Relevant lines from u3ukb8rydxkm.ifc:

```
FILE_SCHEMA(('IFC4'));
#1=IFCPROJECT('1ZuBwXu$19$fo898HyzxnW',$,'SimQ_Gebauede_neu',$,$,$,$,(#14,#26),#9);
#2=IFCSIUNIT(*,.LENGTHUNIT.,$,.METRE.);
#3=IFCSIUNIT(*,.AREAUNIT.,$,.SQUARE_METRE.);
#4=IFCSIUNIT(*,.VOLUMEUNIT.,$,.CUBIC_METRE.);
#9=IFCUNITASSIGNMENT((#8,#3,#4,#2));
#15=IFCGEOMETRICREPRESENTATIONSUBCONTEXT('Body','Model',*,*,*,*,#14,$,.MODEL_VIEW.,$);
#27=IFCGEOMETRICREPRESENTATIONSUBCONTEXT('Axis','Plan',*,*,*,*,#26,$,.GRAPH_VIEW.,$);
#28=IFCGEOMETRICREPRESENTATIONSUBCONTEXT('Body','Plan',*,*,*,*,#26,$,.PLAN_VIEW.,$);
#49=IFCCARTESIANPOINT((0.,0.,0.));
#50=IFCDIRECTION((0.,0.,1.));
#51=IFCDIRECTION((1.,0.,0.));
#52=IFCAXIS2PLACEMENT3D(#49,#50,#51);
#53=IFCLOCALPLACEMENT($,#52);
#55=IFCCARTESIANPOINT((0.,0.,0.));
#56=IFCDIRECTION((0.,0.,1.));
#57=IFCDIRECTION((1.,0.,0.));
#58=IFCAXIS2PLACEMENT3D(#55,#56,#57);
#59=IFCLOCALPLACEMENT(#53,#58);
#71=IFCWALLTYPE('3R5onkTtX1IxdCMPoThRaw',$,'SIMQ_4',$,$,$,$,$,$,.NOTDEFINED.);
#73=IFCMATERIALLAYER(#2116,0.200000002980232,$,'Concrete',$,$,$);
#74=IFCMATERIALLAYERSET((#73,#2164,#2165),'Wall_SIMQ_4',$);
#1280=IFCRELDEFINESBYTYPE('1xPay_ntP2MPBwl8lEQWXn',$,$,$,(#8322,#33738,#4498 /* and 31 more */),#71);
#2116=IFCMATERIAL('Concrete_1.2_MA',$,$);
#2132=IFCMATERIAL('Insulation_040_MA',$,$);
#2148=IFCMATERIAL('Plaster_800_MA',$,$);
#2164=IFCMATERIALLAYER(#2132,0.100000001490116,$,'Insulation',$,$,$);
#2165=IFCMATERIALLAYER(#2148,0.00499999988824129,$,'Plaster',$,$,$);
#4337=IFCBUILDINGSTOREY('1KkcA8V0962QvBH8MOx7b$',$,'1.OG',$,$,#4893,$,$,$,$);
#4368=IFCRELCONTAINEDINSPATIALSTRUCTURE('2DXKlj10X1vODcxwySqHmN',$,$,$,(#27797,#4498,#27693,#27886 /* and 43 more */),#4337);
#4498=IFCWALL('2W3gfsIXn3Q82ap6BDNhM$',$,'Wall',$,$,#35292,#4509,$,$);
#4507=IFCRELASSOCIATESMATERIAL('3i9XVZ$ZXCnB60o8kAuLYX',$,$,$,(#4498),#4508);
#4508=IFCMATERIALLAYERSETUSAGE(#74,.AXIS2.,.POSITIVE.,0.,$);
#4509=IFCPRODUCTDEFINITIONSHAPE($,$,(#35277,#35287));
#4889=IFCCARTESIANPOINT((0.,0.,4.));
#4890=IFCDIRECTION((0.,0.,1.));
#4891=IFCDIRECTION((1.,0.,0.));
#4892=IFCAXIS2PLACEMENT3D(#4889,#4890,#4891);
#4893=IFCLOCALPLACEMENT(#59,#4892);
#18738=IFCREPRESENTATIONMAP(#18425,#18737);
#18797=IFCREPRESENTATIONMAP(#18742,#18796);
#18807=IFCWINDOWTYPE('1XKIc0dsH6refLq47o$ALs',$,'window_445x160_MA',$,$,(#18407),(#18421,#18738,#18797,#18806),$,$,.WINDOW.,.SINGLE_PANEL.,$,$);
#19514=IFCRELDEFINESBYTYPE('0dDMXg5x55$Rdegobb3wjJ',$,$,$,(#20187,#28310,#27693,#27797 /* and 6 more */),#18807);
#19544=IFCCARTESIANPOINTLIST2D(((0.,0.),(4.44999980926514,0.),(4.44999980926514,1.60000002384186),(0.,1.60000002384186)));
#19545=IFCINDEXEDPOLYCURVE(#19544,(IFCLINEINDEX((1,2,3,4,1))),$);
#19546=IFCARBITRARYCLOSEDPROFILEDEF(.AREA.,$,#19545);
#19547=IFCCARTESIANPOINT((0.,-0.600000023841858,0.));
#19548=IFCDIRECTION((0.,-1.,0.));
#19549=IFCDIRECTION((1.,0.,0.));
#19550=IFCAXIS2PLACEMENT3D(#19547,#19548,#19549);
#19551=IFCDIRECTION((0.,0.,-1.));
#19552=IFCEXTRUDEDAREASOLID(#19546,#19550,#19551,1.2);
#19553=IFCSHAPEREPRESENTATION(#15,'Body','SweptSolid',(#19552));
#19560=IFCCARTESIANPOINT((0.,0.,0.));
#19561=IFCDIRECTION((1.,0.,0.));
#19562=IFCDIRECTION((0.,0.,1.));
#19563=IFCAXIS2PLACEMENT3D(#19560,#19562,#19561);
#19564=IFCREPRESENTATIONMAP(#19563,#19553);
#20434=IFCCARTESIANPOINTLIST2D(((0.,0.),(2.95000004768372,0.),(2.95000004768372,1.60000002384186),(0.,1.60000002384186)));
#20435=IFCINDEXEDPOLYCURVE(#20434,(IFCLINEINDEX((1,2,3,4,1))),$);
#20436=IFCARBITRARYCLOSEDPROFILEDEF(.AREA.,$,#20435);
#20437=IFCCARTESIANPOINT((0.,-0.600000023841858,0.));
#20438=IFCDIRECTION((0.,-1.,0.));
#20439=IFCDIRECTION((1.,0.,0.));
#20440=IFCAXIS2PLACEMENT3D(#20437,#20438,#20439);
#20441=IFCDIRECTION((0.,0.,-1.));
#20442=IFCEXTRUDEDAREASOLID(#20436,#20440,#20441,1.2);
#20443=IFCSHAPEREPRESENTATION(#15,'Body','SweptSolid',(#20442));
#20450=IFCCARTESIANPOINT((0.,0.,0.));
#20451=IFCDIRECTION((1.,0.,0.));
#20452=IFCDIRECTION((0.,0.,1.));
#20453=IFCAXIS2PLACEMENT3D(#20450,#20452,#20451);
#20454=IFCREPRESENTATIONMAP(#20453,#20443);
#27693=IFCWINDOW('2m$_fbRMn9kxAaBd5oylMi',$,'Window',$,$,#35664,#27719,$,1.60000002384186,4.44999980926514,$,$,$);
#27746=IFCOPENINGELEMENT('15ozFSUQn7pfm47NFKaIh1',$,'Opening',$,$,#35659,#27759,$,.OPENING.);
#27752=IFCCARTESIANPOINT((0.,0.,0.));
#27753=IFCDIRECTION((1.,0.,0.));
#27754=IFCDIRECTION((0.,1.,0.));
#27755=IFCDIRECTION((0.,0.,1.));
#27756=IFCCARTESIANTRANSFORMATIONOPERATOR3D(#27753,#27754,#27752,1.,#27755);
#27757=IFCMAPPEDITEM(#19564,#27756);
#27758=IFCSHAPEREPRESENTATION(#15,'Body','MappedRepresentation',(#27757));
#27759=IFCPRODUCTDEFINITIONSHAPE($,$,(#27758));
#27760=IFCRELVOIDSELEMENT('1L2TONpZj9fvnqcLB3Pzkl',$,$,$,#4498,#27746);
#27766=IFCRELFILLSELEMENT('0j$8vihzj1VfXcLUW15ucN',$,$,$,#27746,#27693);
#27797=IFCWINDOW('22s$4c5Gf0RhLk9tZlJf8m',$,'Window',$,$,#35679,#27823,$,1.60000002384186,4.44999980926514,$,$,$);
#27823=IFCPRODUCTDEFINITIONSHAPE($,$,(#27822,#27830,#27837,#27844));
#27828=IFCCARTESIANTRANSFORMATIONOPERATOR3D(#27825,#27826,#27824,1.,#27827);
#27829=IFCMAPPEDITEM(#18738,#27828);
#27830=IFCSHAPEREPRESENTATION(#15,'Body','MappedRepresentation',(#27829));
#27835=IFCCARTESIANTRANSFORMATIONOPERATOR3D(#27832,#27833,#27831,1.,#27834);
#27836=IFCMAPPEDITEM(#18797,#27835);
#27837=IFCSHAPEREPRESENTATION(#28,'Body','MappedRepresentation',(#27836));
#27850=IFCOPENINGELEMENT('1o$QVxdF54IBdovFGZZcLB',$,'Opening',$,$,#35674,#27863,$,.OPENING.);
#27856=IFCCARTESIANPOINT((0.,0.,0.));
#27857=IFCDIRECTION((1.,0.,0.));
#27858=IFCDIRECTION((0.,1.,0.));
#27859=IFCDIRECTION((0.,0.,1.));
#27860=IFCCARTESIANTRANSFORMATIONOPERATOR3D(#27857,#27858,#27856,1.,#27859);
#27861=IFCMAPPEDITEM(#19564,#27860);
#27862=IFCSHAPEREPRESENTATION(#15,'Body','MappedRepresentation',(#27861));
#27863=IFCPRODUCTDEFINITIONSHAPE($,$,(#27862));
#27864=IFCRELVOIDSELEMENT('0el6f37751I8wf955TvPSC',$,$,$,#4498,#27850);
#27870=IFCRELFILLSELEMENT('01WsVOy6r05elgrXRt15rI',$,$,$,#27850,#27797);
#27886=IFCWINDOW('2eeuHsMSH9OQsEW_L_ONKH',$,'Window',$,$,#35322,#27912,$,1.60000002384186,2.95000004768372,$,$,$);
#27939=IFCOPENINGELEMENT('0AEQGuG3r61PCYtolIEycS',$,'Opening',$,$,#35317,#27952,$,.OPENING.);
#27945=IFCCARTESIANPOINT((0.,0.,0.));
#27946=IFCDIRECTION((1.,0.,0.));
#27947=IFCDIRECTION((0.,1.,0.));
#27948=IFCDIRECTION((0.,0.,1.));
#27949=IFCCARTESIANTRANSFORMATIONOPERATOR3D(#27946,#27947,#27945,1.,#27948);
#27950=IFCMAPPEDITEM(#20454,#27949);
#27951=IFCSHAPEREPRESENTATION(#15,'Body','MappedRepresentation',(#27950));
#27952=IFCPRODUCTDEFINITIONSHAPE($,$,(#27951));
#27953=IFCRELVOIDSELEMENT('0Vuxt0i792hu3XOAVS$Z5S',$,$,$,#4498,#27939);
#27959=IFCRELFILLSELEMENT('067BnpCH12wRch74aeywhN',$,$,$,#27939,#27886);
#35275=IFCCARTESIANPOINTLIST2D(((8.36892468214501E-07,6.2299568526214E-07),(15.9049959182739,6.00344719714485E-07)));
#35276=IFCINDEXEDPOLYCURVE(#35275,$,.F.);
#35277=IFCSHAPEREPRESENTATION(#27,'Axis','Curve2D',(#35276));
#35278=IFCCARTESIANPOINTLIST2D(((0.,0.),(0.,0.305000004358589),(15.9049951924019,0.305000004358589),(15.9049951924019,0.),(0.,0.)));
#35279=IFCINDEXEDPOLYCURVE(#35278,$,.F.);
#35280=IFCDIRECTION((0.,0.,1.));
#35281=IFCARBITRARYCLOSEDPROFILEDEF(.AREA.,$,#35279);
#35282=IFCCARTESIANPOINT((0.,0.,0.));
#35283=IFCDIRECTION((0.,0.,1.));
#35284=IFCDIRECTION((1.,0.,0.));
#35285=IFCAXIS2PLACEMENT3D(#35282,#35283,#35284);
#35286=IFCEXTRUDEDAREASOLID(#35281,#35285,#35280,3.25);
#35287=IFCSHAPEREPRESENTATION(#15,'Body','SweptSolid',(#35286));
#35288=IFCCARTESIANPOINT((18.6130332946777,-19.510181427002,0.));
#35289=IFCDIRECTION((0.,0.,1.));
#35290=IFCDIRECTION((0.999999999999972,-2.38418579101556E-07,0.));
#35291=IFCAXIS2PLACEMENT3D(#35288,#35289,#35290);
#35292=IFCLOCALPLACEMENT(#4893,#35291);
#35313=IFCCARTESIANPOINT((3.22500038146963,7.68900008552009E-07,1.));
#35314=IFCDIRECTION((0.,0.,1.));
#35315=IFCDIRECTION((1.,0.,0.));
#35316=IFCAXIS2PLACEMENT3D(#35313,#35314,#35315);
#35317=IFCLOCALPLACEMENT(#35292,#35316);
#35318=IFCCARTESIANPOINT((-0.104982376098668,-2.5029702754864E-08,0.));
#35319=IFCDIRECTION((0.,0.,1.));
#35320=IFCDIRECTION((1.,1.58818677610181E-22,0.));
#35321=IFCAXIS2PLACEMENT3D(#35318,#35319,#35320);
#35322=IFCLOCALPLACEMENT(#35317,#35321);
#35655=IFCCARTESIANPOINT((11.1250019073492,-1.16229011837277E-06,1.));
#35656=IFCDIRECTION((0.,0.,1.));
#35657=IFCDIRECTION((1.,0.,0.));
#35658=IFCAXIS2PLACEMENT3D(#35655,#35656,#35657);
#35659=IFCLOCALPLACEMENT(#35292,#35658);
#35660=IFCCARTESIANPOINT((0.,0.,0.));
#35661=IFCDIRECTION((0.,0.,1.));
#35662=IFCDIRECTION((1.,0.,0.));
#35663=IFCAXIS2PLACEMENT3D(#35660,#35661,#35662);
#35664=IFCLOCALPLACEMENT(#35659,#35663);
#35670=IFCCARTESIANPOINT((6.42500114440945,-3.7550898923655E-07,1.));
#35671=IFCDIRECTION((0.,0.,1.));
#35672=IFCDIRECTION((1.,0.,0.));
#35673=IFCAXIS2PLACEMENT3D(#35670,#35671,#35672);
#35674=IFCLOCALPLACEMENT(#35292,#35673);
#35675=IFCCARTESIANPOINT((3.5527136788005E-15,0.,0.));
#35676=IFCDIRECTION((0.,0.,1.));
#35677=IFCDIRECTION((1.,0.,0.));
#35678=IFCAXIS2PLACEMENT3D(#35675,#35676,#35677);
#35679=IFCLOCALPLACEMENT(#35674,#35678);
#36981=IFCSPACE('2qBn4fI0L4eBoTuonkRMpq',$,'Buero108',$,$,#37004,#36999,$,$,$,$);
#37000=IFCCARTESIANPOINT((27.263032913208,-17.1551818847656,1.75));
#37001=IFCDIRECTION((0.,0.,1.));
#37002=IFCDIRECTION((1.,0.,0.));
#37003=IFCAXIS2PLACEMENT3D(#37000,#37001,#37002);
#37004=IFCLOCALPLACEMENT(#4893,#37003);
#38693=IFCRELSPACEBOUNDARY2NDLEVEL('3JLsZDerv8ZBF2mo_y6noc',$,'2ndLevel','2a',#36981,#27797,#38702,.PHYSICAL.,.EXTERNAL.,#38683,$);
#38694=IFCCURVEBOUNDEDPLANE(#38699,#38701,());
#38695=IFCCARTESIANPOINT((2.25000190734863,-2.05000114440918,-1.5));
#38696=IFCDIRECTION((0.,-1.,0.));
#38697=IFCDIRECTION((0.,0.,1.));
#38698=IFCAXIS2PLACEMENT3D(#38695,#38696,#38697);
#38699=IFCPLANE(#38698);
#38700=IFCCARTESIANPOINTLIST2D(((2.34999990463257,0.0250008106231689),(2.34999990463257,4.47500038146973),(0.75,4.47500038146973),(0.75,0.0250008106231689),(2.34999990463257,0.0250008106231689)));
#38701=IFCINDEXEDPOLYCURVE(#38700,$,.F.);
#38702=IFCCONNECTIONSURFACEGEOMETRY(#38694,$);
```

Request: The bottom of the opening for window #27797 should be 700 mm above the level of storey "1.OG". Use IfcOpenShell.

```python
import numpy as np
import ifcopenshell
import ifcopenshell.api.geometry
import ifcopenshell.geom
import ifcopenshell.util.element
import ifcopenshell.util.placement
import ifcopenshell.util.shape
import ifcopenshell.util.unit

model = ifcopenshell.open("u3ukb8rydxkm.ifc")
unit_scale = ifcopenshell.util.unit.calculate_unit_scale(model)

window = model.by_guid("22s$4c5Gf0RhLk9tZlJf8m")
opening = window.FillsVoids[0].RelatingOpeningElement
storey = ifcopenshell.util.element.get_container(window, ifc_class="IfcBuildingStorey")
level = ifcopenshell.util.placement.get_local_placement(storey.ObjectPlacement)[2, 3]

# The opening's origin need not be at the sill, so measure its lowest point.
shape = ifcopenshell.geom.create_shape(ifcopenshell.geom.settings(), opening)
bottom = ifcopenshell.util.shape.get_shape_bottom_elevation(shape, shape.geometry) / unit_scale
dz = level + 0.7 - bottom

shift = np.array([0.0, 0.0, dz])
# The window is placed relative to its opening, so it follows when the opening moves.
matrix = ifcopenshell.util.placement.get_local_placement(opening.ObjectPlacement)
matrix[:3, 3] += shift
ifcopenshell.api.geometry.edit_object_placement(
    model, product=opening, matrix=matrix, is_si=False, should_transform_children=True
)

# Space boundary surfaces are stored in each space's coordinates; move them too.
for rel in window.ProvidesBoundaries:
    if not rel.ConnectionGeometry:
        continue
    surface = rel.ConnectionGeometry.SurfaceOnRelatingElement.BasisSurface
    space_matrix = ifcopenshell.util.placement.get_local_placement(rel.RelatingSpace.ObjectPlacement)
    point = np.array(surface.Position.Location.Coordinates) + space_matrix[:3, :3].T @ shift
    surface.Position = model.createIfcAxis2Placement3D(
        model.createIfcCartesianPoint(point.tolist()), surface.Position.Axis, surface.Position.RefDirection
    )

print(f"moved by {dz * unit_scale:+.3f} m")

model.write("u3ukb8rydxkm_edited.ifc")
```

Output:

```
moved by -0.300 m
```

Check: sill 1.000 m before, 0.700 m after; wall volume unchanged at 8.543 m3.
